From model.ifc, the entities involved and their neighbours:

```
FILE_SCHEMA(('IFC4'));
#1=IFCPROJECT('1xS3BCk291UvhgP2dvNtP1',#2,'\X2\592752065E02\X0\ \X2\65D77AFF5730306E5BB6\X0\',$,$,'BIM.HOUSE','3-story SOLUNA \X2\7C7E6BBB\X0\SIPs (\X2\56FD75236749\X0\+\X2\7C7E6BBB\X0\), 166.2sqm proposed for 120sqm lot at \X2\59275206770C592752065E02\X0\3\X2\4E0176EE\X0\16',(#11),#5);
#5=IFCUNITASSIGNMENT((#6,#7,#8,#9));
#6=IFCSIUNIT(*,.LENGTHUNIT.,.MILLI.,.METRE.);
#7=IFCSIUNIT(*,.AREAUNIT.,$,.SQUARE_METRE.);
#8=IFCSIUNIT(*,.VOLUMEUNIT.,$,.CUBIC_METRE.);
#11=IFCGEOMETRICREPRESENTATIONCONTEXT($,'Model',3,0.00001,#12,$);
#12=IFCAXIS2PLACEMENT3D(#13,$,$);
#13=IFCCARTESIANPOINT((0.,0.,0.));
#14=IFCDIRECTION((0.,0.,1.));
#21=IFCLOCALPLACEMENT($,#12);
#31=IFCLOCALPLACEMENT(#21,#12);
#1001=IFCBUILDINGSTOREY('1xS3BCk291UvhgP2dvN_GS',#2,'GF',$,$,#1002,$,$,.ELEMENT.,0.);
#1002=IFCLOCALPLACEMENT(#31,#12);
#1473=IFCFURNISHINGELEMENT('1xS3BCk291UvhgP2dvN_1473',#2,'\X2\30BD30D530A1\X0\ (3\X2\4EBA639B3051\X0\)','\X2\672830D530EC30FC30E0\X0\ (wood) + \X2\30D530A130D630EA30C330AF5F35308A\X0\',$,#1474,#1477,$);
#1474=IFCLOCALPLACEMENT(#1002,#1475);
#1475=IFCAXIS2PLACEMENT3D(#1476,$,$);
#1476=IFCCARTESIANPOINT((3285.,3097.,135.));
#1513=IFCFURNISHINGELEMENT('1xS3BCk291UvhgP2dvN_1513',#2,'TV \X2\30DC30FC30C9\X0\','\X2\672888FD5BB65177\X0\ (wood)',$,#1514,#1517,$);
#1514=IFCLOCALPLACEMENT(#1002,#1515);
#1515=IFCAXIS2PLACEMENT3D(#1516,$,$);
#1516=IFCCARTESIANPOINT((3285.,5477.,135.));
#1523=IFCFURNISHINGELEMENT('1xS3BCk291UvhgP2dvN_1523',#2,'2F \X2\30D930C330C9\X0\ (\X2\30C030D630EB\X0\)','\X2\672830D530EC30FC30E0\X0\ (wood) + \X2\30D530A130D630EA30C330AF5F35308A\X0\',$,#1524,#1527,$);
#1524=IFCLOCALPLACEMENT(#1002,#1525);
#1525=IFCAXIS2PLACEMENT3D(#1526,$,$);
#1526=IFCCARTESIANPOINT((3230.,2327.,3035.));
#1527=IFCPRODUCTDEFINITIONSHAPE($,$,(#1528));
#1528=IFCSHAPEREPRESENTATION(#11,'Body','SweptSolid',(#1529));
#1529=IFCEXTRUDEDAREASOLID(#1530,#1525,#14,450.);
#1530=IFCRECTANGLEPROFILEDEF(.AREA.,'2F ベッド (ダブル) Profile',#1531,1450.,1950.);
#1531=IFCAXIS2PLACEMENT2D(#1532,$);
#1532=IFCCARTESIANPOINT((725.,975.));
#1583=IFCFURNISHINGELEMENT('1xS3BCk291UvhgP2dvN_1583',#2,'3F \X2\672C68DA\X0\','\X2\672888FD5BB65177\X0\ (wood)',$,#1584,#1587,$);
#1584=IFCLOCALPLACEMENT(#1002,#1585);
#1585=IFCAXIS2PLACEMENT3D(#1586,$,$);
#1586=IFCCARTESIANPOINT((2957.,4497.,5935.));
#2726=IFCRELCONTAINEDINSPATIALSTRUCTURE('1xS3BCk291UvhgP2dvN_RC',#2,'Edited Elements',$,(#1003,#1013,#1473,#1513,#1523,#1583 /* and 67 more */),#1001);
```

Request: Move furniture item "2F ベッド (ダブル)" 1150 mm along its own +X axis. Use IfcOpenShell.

```python
import ifcopenshell
import ifcopenshell.api.geometry
import ifcopenshell.util.placement

model = ifcopenshell.open("model.ifc")

item = model.by_guid("1xS3BCk291UvhgP2dvN_1523")
matrix = ifcopenshell.util.placement.get_local_placement(item.ObjectPlacement)
matrix[:3, 3] += matrix[:3, 0] * 1150.0
ifcopenshell.api.geometry.edit_object_placement(model, product=item, matrix=matrix, is_si=False)

print(ifcopenshell.util.placement.get_local_placement(item.ObjectPlacement).round(3) + 0.0)

model.write("model-out.ifc")
```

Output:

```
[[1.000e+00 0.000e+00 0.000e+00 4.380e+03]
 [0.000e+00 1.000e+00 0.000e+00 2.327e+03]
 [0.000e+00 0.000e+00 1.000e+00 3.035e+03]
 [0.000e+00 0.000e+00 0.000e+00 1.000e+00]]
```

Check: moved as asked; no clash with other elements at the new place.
